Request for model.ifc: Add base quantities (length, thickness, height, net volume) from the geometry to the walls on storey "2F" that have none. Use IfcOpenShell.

First a look at what the model holds.

```python
import ifcopenshell
import ifcopenshell.util.element
import ifcopenshell.util.unit

model = ifcopenshell.open("model.ifc")
print(model.schema)
for unit_type in ("LENGTHUNIT", "AREAUNIT", "VOLUMEUNIT"):
    print(unit_type, ifcopenshell.util.unit.calculate_unit_scale(model, unit_type))
storey = next(s for s in model.by_type("IfcBuildingStorey") if s.Name == "2F")
walls = [e for e in ifcopenshell.util.element.get_decomposition(storey) if e.is_a("IfcWall")]
for e in sorted(walls, key=lambda e: e.id()):
    print(e.id(), e.is_a(), e.Name, list(ifcopenshell.util.element.get_psets(e, qtos_only=True)), sep=" | ")
```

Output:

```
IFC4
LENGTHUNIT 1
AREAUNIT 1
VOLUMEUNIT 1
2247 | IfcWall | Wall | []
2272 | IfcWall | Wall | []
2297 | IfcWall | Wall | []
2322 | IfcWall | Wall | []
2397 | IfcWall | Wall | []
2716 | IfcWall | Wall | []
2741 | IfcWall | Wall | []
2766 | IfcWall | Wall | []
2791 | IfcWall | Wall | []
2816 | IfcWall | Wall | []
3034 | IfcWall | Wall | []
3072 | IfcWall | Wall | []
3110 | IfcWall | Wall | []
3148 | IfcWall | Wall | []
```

```python
import ifcopenshell
import ifcopenshell.api.pset
import ifcopenshell.geom
import ifcopenshell.util.element
import ifcopenshell.util.shape
import ifcopenshell.util.unit

model = ifcopenshell.open("model.ifc")
unit_scale = ifcopenshell.util.unit.calculate_unit_scale(model)
volume_scale = ifcopenshell.util.unit.calculate_unit_scale(model, "VOLUMEUNIT")
settings = ifcopenshell.geom.settings()

storey = next(s for s in model.by_type("IfcBuildingStorey") if s.Name == "2F")
walls = [e for e in ifcopenshell.util.element.get_decomposition(storey) if e.is_a("IfcWall")]

for e in sorted(walls, key=lambda e: e.id()):
    if ifcopenshell.util.element.get_psets(e, qtos_only=True, should_inherit=False):
        continue
    # Geometry comes back in metres, in the element's own axes.
    shape = ifcopenshell.geom.create_shape(settings, e)
    values = {
        "Length": ifcopenshell.util.shape.get_x(shape.geometry) / unit_scale,
        "Width": ifcopenshell.util.shape.get_y(shape.geometry) / unit_scale,
        "Height": ifcopenshell.util.shape.get_z(shape.geometry) / unit_scale,
        "NetVolume": ifcopenshell.util.shape.get_volume(shape.geometry) / volume_scale,
    }
    qto = ifcopenshell.api.pset.add_qto(model, product=e, name="Qto_WallBaseQuantities")
    ifcopenshell.api.pset.edit_qto(model, qto=qto, properties=values)
    print(e.id(), {k: round(v, 3) for k, v in values.items()})

model.write("model-out.ifc")
```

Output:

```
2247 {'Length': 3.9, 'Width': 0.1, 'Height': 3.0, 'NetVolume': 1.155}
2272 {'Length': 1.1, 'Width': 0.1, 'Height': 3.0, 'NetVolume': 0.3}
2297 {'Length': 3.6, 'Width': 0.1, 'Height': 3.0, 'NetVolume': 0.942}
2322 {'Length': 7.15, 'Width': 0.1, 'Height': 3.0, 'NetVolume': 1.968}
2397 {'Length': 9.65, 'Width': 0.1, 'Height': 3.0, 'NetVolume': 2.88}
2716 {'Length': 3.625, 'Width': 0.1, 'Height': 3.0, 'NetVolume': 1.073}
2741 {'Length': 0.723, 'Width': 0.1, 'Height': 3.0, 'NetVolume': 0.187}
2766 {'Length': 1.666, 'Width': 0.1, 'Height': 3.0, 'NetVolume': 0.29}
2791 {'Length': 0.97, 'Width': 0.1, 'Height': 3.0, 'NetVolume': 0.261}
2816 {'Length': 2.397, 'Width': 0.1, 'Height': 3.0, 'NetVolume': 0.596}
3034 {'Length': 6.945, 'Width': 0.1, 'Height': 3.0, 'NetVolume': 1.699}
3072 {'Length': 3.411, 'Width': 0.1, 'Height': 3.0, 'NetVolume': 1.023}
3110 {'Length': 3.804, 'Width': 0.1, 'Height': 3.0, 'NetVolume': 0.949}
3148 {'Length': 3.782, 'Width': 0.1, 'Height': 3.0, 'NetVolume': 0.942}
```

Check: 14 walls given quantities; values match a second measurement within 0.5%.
